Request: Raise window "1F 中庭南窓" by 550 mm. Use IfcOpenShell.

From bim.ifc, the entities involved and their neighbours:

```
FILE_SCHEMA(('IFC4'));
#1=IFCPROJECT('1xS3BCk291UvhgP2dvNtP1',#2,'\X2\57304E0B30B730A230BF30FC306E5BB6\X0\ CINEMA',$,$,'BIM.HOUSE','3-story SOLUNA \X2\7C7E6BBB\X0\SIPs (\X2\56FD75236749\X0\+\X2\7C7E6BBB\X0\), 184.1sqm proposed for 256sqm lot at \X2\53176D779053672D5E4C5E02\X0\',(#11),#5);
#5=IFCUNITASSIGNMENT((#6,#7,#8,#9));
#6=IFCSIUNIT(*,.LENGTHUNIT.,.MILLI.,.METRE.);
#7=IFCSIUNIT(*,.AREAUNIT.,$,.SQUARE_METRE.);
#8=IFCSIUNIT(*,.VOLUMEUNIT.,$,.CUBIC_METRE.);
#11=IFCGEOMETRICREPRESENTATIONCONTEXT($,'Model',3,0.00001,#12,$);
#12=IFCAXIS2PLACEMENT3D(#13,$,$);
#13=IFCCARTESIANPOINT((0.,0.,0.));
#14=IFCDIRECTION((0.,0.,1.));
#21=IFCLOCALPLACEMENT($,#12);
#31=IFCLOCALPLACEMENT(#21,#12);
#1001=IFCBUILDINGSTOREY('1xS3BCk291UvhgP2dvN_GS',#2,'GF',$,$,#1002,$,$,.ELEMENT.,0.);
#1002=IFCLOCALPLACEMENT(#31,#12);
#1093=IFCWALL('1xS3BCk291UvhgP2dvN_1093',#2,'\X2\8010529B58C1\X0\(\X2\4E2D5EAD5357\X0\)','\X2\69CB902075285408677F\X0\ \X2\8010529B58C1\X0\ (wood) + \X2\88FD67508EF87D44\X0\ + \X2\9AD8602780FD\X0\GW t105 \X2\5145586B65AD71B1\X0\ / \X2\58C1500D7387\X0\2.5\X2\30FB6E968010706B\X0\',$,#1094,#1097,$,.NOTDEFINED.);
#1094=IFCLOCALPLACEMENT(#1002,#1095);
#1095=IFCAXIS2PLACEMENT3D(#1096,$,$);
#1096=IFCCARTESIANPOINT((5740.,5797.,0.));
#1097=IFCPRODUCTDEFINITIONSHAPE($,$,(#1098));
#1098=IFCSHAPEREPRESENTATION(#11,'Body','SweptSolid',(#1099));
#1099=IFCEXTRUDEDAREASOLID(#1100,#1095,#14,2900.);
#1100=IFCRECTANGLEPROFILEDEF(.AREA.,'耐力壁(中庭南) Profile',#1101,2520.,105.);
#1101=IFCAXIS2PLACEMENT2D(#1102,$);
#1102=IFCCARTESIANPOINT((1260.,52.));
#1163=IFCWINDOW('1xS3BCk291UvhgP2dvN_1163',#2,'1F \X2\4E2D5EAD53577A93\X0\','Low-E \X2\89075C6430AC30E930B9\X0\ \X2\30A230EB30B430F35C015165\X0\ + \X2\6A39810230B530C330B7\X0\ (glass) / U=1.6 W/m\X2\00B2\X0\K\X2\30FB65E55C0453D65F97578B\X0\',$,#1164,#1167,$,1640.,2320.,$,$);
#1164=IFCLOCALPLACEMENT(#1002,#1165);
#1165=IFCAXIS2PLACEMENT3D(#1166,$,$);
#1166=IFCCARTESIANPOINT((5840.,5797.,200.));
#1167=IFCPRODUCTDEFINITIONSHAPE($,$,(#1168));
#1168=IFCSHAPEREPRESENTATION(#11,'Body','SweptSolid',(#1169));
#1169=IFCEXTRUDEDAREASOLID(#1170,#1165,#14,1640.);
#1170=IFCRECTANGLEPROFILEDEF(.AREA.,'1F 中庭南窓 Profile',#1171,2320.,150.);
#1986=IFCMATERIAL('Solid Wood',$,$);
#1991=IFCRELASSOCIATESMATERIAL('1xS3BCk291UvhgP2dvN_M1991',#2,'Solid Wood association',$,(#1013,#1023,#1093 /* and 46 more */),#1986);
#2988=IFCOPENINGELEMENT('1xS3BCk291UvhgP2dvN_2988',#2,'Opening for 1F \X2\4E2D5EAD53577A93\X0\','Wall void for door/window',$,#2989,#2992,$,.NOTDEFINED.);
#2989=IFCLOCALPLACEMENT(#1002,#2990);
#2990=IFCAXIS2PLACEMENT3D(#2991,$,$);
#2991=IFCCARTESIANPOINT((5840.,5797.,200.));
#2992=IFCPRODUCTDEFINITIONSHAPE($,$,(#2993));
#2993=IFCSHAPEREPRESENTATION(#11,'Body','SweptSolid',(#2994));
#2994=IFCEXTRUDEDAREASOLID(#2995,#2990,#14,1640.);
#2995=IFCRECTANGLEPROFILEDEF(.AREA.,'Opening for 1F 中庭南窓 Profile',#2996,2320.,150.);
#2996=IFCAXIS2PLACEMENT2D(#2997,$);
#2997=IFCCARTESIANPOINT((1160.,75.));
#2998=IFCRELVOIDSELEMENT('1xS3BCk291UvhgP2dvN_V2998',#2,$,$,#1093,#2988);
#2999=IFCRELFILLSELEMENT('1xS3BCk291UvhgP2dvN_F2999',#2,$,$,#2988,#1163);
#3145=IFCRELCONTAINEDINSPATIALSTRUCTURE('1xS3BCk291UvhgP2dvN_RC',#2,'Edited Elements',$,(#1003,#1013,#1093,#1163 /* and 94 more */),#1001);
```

```python
import numpy as np
import ifcopenshell
import ifcopenshell.api.geometry
import ifcopenshell.util.placement
import ifcopenshell.util.unit

model = ifcopenshell.open("bim.ifc")
unit_scale = ifcopenshell.util.unit.calculate_unit_scale(model)

window = model.by_id(1163)
opening = window.FillsVoids[0].RelatingOpeningElement
dz = 550.0

shift = np.array([0.0, 0.0, dz])
# The window is not placed relative to its opening, so move both.
for product in (opening, window):
    matrix = ifcopenshell.util.placement.get_local_placement(product.ObjectPlacement)
    matrix[:3, 3] += shift
    ifcopenshell.api.geometry.edit_object_placement(model, product=product, matrix=matrix, is_si=False)

print(f"moved by {dz * unit_scale:+.3f} m")

model.write("bim_v2.ifc")
```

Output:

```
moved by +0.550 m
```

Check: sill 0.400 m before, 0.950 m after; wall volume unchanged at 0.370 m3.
